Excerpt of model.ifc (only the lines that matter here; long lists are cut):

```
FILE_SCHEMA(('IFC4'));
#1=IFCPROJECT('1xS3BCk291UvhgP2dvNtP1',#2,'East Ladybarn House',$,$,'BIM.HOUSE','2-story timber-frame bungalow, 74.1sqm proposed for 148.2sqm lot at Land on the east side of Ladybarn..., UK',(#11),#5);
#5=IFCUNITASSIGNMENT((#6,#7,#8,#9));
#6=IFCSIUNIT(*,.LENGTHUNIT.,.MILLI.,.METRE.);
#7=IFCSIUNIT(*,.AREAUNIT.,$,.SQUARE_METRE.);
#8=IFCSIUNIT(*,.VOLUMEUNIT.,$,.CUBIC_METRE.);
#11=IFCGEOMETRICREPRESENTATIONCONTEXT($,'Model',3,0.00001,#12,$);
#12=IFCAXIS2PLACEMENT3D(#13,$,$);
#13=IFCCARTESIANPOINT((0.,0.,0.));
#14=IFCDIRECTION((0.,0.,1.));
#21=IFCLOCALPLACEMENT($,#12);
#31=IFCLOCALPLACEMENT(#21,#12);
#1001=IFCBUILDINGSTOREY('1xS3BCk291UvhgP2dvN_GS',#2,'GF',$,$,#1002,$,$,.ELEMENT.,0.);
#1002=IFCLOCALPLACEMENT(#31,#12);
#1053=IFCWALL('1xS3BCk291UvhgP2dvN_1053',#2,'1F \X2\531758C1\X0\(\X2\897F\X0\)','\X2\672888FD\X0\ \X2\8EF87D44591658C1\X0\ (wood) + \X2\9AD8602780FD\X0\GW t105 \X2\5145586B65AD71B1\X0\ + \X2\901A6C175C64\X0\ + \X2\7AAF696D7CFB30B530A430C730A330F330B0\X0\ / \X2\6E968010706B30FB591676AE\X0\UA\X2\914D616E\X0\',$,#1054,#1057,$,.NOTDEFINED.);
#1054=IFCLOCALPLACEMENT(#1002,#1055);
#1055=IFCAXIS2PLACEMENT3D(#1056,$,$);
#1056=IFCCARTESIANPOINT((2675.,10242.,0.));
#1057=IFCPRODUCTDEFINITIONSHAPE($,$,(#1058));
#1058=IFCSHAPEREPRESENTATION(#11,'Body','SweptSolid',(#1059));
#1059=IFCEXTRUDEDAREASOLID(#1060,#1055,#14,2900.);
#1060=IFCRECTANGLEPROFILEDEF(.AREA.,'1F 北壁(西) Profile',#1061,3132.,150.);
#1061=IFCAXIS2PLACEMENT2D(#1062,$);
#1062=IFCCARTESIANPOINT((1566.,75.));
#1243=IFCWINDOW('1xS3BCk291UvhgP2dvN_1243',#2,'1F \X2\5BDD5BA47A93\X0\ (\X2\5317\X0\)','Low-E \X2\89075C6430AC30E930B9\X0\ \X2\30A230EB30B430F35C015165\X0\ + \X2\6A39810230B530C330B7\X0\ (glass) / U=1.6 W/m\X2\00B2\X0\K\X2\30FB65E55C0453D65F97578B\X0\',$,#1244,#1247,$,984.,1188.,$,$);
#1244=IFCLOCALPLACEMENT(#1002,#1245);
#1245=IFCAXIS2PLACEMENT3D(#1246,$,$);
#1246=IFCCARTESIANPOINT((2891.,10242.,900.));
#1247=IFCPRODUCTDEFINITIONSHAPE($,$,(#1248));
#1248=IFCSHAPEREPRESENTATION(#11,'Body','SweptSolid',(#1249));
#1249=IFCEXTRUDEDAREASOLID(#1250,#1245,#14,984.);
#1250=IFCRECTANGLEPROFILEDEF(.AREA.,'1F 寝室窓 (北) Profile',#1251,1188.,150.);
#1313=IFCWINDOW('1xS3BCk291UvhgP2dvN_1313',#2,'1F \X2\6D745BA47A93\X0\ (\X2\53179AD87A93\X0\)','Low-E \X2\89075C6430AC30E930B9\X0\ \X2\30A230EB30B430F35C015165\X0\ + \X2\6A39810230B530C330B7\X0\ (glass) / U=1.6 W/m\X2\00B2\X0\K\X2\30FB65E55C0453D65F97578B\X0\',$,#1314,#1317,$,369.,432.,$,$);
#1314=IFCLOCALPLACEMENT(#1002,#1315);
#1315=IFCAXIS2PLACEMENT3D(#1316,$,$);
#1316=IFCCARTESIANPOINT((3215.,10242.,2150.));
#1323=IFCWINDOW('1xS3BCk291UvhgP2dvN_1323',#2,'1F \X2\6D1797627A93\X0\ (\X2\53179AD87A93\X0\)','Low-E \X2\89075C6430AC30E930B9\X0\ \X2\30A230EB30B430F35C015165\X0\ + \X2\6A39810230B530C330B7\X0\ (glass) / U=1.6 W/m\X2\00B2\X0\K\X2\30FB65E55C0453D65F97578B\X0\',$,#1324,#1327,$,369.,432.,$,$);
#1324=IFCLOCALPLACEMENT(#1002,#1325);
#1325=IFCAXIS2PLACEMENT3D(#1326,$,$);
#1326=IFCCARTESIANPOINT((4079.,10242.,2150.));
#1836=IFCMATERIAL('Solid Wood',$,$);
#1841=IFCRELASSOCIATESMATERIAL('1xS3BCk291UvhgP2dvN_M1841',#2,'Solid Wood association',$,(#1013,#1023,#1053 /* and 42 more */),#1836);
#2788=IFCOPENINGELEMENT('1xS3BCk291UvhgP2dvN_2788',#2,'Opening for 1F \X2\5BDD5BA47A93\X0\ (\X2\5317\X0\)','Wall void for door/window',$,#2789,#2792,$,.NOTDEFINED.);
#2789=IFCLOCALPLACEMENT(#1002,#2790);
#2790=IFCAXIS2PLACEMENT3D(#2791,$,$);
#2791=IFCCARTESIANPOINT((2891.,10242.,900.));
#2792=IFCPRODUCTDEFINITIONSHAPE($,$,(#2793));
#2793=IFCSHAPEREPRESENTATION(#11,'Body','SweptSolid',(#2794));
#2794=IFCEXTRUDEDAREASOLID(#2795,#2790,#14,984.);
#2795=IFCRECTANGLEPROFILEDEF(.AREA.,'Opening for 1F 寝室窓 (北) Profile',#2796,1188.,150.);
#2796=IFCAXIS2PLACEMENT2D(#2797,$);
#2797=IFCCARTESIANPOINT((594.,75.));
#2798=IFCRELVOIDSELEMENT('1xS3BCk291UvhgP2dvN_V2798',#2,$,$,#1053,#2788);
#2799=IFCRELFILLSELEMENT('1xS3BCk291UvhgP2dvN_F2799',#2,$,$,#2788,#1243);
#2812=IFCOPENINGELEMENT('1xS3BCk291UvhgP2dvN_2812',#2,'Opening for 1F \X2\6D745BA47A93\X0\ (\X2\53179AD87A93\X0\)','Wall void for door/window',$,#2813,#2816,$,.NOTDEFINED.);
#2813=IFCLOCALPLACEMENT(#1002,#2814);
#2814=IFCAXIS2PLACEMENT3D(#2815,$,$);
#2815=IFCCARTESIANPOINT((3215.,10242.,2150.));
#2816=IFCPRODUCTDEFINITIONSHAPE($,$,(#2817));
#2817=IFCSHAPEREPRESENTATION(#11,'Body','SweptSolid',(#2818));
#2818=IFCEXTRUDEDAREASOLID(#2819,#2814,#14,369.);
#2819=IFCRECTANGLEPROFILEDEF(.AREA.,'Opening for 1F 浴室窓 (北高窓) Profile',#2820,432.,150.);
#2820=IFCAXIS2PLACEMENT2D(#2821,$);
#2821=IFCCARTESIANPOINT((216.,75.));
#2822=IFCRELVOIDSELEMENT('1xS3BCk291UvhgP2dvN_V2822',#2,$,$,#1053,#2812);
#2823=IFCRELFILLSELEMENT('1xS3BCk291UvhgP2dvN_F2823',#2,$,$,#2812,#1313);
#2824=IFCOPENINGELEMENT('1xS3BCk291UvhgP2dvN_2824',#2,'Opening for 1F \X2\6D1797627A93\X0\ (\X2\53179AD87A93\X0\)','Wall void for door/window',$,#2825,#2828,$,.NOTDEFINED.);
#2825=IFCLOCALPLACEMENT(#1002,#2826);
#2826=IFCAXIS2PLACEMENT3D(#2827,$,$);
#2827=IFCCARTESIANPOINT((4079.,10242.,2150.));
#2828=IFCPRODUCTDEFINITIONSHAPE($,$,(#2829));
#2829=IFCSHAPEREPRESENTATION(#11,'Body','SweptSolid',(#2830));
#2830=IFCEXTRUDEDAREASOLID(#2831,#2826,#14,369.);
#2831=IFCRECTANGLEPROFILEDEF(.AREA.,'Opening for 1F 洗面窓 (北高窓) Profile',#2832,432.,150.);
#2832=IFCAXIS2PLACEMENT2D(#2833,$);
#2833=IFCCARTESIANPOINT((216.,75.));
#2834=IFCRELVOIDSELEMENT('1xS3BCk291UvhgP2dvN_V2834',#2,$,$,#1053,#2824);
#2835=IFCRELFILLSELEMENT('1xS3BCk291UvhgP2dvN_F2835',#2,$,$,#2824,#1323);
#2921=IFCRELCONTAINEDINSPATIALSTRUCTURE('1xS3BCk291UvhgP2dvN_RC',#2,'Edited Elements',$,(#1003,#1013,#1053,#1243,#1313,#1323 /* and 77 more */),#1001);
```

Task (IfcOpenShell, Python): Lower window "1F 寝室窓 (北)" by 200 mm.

```python
import numpy as np
import ifcopenshell
import ifcopenshell.api.geometry
import ifcopenshell.util.placement
import ifcopenshell.util.unit

model = ifcopenshell.open("model.ifc")
unit_scale = ifcopenshell.util.unit.calculate_unit_scale(model)

window = model.by_guid("1xS3BCk291UvhgP2dvN_1243")
opening = window.FillsVoids[0].RelatingOpeningElement
dz = -200.0

shift = np.array([0.0, 0.0, dz])
# The window is not placed relative to its opening, so move both.
for product in (opening, window):
    matrix = ifcopenshell.util.placement.get_local_placement(product.ObjectPlacement)
    matrix[:3, 3] += shift
    ifcopenshell.api.geometry.edit_object_placement(model, product=product, matrix=matrix, is_si=False)

print(f"moved by {dz * unit_scale:+.3f} m")

model.write("model_edited.ifc")
```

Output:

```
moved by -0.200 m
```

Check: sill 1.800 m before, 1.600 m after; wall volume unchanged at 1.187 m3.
